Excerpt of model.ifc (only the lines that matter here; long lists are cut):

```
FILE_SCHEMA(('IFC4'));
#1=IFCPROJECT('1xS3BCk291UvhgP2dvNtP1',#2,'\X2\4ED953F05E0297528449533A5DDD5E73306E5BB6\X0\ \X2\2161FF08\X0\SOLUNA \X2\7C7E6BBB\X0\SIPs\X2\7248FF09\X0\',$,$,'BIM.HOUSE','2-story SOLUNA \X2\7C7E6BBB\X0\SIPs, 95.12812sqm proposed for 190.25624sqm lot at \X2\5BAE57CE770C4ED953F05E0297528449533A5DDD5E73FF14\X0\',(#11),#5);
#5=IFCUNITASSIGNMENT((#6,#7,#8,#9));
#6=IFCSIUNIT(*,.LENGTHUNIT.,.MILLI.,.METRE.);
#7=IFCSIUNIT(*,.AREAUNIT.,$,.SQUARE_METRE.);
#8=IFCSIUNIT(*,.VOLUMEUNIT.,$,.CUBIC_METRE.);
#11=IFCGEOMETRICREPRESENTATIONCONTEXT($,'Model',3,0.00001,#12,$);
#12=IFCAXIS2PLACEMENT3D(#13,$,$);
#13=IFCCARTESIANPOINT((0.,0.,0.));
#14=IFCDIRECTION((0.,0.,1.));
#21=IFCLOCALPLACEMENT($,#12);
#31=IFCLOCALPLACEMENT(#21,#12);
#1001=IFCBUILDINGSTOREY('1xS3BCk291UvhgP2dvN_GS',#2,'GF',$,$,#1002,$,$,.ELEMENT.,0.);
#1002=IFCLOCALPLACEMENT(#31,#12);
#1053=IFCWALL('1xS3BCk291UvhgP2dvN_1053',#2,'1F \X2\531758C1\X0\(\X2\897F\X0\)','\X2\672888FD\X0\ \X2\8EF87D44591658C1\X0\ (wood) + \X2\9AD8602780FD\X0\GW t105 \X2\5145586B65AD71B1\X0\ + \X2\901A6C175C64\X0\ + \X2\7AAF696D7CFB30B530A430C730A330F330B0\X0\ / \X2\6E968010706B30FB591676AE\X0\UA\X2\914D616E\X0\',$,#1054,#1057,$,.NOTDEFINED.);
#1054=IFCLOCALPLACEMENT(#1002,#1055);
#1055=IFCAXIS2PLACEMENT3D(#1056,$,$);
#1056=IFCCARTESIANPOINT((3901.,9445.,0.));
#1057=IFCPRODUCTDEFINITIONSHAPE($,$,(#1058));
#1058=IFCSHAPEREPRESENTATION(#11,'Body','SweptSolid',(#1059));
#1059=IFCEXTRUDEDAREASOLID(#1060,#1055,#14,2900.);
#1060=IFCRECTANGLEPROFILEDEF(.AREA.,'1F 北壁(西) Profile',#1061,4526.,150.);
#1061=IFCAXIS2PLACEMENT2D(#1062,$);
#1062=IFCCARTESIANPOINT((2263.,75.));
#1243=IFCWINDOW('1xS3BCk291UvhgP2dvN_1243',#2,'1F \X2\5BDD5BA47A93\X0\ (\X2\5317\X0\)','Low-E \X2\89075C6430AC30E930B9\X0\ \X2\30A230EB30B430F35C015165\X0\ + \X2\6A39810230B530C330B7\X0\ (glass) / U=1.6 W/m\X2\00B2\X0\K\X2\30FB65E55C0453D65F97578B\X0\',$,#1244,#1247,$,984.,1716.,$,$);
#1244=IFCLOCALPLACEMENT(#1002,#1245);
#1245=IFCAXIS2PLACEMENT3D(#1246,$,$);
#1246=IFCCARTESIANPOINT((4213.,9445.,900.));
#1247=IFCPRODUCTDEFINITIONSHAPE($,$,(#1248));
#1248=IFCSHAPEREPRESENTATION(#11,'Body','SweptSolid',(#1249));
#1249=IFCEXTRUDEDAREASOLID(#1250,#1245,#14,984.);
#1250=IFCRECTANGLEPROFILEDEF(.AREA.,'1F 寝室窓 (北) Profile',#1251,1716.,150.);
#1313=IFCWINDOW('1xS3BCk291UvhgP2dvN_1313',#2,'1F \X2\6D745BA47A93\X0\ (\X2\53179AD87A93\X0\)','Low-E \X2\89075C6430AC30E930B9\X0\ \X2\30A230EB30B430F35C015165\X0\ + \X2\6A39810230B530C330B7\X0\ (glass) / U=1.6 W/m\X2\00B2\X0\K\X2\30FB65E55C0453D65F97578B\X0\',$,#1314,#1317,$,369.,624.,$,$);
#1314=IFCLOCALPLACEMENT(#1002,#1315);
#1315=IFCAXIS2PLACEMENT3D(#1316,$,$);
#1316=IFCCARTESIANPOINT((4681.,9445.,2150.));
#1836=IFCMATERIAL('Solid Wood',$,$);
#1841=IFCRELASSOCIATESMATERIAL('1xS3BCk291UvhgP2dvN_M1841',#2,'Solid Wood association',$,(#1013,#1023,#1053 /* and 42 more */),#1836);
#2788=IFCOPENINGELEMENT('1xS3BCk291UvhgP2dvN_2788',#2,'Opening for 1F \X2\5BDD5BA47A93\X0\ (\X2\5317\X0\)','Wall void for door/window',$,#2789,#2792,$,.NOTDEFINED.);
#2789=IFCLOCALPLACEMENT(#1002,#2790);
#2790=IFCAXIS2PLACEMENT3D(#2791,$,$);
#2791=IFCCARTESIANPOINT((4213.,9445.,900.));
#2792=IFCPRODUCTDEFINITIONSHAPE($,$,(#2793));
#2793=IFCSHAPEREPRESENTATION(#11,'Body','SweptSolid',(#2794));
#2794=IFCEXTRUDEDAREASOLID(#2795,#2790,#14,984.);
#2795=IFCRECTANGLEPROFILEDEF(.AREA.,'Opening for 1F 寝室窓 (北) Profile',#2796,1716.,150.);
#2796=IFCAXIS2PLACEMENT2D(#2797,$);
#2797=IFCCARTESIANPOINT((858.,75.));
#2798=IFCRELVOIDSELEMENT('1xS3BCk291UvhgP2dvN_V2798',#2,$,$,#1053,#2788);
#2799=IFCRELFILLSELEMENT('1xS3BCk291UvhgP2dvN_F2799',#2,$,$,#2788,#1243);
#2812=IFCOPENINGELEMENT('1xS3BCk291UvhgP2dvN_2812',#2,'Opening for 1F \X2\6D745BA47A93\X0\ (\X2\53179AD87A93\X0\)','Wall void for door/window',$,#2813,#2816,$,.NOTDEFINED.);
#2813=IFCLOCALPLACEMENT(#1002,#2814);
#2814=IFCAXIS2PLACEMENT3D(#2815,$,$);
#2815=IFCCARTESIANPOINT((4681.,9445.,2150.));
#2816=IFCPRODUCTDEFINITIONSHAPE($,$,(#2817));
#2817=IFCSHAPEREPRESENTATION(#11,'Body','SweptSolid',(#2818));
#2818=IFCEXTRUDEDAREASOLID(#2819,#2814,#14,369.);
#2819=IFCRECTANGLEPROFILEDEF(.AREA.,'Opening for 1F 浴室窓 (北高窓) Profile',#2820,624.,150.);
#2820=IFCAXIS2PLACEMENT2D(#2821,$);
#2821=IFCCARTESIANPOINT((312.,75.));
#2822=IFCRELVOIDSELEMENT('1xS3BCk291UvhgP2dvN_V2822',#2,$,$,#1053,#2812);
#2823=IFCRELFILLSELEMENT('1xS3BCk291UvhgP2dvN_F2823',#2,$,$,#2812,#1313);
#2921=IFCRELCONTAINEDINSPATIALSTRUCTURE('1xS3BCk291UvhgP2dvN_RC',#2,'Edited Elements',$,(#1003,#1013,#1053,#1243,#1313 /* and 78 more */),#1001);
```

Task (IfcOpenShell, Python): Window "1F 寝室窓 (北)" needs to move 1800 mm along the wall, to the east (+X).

```python
import ifcopenshell
import ifcopenshell.api.geometry
import ifcopenshell.util.placement

model = ifcopenshell.open("model.ifc")

window = model.by_guid("1xS3BCk291UvhgP2dvN_1243")
opening = window.FillsVoids[0].RelatingOpeningElement
wall = opening.VoidsElements[0].RelatingBuildingElement

wall_matrix = ifcopenshell.util.placement.get_local_placement(wall.ObjectPlacement)
shift = wall_matrix[:3, 0] * 1800.0
before = ifcopenshell.util.placement.get_local_placement(window.ObjectPlacement)[:3, 3].copy()

# The window is not placed relative to its opening, so move both.
for product in (opening, window):
    matrix = ifcopenshell.util.placement.get_local_placement(product.ObjectPlacement)
    matrix[:3, 3] += shift
    ifcopenshell.api.geometry.edit_object_placement(model, product=product, matrix=matrix, is_si=False)

after = ifcopenshell.util.placement.get_local_placement(window.ObjectPlacement)[:3, 3]
print("window moved by", (after - before).round(3) + 0.0)

model.write("model_v2.ifc")
```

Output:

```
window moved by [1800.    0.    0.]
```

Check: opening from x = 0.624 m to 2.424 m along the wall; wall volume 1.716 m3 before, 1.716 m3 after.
